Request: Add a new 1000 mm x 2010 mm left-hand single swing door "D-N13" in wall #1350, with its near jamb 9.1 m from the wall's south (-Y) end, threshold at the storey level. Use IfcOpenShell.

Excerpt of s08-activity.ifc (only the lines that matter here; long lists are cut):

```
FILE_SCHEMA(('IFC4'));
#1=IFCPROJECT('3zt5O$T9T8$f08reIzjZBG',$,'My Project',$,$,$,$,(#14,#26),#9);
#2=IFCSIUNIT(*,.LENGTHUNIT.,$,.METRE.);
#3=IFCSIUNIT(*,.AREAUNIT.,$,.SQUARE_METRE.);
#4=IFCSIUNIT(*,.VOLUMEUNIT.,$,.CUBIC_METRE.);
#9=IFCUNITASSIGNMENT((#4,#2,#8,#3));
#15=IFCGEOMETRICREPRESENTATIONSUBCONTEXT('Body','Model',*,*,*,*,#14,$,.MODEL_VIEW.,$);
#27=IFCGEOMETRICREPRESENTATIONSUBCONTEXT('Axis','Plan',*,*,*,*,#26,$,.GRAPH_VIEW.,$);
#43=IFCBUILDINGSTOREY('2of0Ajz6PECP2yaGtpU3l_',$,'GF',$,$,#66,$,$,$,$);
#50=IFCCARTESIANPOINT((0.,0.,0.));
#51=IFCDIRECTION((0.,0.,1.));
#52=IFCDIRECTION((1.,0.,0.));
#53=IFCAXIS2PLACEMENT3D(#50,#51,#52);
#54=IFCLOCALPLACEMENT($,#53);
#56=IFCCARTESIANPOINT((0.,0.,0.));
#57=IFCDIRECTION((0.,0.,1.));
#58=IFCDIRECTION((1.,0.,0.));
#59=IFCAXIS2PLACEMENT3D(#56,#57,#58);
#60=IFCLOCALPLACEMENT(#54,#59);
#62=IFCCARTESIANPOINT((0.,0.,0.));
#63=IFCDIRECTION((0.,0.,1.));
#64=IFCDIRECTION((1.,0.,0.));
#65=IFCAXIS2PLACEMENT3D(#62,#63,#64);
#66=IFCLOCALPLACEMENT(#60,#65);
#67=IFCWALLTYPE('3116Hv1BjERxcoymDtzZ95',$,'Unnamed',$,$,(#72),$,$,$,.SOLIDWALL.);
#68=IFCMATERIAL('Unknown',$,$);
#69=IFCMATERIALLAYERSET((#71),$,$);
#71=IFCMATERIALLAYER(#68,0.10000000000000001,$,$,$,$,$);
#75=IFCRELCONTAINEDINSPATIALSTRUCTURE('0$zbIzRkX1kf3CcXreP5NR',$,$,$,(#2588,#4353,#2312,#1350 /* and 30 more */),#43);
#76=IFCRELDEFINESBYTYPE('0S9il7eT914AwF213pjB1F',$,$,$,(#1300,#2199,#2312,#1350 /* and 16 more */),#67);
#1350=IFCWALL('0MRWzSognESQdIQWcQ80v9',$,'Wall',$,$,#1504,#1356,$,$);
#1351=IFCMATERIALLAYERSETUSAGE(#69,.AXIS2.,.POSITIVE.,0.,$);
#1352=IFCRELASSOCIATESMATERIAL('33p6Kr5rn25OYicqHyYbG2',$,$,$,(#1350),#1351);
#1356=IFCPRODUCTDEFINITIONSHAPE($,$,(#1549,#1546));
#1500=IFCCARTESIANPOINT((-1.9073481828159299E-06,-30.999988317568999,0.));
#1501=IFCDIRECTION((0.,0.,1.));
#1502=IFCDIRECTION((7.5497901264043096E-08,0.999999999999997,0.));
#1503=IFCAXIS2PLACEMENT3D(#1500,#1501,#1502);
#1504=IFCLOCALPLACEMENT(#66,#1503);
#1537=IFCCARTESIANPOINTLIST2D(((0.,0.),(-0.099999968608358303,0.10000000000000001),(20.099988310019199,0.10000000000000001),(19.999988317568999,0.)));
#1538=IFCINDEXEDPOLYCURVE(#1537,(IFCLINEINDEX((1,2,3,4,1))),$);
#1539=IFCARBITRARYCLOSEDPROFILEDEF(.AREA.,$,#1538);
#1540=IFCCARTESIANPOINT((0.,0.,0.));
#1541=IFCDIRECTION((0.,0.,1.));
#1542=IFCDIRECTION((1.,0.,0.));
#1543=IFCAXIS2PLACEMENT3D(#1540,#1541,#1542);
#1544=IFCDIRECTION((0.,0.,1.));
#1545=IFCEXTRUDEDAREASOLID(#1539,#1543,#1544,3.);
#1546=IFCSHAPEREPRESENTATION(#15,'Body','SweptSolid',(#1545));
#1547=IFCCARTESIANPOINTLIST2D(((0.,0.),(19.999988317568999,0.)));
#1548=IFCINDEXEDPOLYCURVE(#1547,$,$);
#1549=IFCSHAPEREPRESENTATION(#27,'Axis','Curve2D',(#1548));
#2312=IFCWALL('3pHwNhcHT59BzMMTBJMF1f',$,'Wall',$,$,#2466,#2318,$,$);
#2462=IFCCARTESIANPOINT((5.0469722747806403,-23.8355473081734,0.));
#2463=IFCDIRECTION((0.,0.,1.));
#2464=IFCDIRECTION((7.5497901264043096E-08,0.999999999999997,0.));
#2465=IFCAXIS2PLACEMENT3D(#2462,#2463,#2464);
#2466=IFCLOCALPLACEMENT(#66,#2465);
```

```python
import numpy as np
import ifcopenshell
import ifcopenshell.api.feature
import ifcopenshell.api.geometry
import ifcopenshell.api.root
import ifcopenshell.api.spatial
import ifcopenshell.geom
import ifcopenshell.util.element
import ifcopenshell.util.placement
import ifcopenshell.util.representation
import ifcopenshell.util.shape
import ifcopenshell.util.unit

model = ifcopenshell.open("s08-activity.ifc")
unit_scale = ifcopenshell.util.unit.calculate_unit_scale(model)
settings = ifcopenshell.geom.settings()


def volume(element):
    """Net volume in cubic metres, openings subtracted."""
    shape = ifcopenshell.geom.create_shape(settings, element)
    return ifcopenshell.util.shape.get_volume(shape.geometry)


wall = model.by_guid("0MRWzSognESQdIQWcQ80v9")
storey = ifcopenshell.util.element.get_container(wall, ifc_class="IfcBuildingStorey")
context = ifcopenshell.util.representation.get_context(model, "Model", "Body", "MODEL_VIEW")
before = volume(wall)

width, height, from_end, sill = 1, 2.01, 9.1, 0.0  # metres

# The wall runs along its own X axis, and the end named is its -X end.
wall_shape = ifcopenshell.geom.create_shape(settings, wall)
x, y, z = ifcopenshell.util.shape.get_vertices(wall_shape.geometry).T
start = x.min() + from_end
face, thickness = float(y.min()), float(y.max() - y.min())
wall_matrix = ifcopenshell.util.placement.get_local_placement(wall.ObjectPlacement)
level = ifcopenshell.util.placement.get_local_placement(storey.ObjectPlacement)[2, 3]


def in_wall(x, y):
    """Placement at x, y metres in the wall's axes, at sill height."""
    matrix = wall_matrix.copy()
    matrix[:, 3] = wall_matrix @ np.array([x / unit_scale, y / unit_scale, 0.0, 1.0])
    matrix[2, 3] = level + sill / unit_scale
    return matrix


# Opening: a box that overshoots both wall faces by 50 mm.
opening = ifcopenshell.api.root.create_entity(model, ifc_class="IfcOpeningElement", predefined_type="OPENING")
box = ifcopenshell.api.geometry.add_wall_representation(
    model, context=context, length=width, height=height, thickness=thickness + 0.1
)
ifcopenshell.api.geometry.assign_representation(model, product=opening, representation=box)
ifcopenshell.api.geometry.edit_object_placement(model, product=opening, matrix=in_wall(start, face - 0.05), is_si=False)
ifcopenshell.api.feature.add_feature(model, feature=opening, element=wall)

door = ifcopenshell.api.root.create_entity(model, ifc_class="IfcDoor", name="D-N13", predefined_type="DOOR")
door.OverallWidth, door.OverallHeight = width / unit_scale, height / unit_scale
door.OperationType = "SINGLE_SWING_LEFT"
body = ifcopenshell.api.geometry.add_door_representation(
    model,
    context=context,
    overall_width=door.OverallWidth,
    overall_height=door.OverallHeight,
    operation_type="SINGLE_SWING_LEFT",
    lining_properties={"LiningDepth": thickness / unit_scale, "ThresholdDepth": thickness / unit_scale},
)
ifcopenshell.api.geometry.assign_representation(model, product=door, representation=body)
ifcopenshell.api.spatial.assign_container(model, products=[door], relating_structure=storey)
ifcopenshell.api.feature.add_filling(model, opening=opening, element=door)

# The lining spans the wall, so the door starts at the wall face.
ifcopenshell.api.geometry.edit_object_placement(model, product=door, matrix=in_wall(start, face), is_si=False)

after = volume(wall)

print(f"wall volume {before:.3f} -> {after:.3f} m3")

model.write("s08-activity_edited.ifc")
```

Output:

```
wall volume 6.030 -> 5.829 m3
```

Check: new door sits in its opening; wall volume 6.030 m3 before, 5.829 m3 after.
